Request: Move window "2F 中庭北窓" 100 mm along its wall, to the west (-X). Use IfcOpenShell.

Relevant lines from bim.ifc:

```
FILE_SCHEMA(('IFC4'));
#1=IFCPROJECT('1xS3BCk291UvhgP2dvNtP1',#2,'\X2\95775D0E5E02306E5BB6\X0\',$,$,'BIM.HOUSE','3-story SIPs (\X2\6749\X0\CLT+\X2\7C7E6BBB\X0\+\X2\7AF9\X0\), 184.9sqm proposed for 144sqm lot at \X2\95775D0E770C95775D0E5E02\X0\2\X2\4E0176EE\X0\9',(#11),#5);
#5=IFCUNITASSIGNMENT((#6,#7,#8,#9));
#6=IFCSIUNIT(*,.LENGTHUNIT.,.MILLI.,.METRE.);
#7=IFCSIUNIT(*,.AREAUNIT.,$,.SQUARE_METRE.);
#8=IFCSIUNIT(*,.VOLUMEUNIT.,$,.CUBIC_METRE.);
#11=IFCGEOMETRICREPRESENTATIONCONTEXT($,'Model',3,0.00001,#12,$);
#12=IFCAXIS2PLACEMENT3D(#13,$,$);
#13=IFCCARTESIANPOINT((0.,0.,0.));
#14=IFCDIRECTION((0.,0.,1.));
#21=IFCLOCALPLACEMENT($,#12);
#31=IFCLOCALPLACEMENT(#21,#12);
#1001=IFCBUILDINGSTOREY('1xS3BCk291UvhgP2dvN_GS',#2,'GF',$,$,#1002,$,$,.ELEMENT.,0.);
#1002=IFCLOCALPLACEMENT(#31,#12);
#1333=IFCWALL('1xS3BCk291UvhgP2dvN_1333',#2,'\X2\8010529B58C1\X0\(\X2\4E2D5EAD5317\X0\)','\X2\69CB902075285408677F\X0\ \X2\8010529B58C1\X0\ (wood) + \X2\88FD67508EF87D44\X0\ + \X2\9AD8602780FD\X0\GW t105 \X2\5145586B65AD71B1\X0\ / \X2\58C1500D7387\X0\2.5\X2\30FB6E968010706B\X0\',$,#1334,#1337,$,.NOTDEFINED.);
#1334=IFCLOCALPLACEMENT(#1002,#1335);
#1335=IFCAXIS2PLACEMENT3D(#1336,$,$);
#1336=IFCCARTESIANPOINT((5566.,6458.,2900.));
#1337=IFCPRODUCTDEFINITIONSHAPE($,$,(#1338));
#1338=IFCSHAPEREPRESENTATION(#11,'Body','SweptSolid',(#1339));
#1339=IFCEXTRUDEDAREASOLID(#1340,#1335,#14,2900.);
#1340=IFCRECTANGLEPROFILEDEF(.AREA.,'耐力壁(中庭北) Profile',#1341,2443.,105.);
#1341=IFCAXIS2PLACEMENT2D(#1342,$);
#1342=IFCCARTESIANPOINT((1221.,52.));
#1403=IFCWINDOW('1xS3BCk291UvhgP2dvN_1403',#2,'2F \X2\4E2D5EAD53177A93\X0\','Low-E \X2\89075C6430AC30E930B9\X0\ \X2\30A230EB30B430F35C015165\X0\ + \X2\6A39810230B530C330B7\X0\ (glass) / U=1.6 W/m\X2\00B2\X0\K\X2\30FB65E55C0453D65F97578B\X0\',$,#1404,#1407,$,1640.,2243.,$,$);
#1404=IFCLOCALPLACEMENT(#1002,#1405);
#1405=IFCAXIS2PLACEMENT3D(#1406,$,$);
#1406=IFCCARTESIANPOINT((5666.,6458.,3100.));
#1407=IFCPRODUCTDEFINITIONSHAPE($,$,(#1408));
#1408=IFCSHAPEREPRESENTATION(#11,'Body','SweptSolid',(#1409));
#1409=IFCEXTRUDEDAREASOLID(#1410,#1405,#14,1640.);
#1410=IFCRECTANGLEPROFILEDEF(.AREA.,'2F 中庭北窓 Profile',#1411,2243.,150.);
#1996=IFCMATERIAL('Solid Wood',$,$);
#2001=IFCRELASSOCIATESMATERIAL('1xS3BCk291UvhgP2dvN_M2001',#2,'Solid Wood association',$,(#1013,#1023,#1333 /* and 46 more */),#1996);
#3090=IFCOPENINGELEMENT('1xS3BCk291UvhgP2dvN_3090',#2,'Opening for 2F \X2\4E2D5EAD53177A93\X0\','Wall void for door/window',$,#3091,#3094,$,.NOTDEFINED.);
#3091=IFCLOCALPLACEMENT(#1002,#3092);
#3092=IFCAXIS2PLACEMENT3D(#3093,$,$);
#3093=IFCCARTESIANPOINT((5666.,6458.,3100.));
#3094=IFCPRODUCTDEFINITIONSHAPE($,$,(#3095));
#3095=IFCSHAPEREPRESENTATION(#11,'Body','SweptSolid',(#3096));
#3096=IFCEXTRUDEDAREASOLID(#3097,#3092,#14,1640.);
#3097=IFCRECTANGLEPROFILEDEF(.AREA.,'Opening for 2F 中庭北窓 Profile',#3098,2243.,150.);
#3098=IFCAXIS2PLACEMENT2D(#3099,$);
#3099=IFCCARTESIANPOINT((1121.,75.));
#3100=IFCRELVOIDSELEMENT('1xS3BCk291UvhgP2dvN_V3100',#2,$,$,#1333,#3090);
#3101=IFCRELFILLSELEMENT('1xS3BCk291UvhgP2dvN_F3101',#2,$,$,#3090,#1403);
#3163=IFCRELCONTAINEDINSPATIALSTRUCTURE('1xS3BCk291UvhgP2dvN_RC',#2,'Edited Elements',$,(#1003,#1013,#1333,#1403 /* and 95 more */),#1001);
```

```python
import ifcopenshell
import ifcopenshell.api.geometry
import ifcopenshell.util.placement
import ifcopenshell.util.unit

model = ifcopenshell.open("bim.ifc")
unit_scale = ifcopenshell.util.unit.calculate_unit_scale(model)

window = model.by_guid("1xS3BCk291UvhgP2dvN_1403")
opening = window.FillsVoids[0].RelatingOpeningElement
wall = opening.VoidsElements[0].RelatingBuildingElement

wall_matrix = ifcopenshell.util.placement.get_local_placement(wall.ObjectPlacement)
shift = wall_matrix[:3, 0] * -0.1 / unit_scale
before = ifcopenshell.util.placement.get_local_placement(window.ObjectPlacement)[:3, 3].copy()

# The window is not placed relative to its opening, so move both.
for product in (opening, window):
    matrix = ifcopenshell.util.placement.get_local_placement(product.ObjectPlacement)
    matrix[:3, 3] += shift
    ifcopenshell.api.geometry.edit_object_placement(model, product=product, matrix=matrix, is_si=False)

after = ifcopenshell.util.placement.get_local_placement(window.ObjectPlacement)[:3, 3]
print("window moved by", (after - before).round(3) + 0.0)

model.write("bim_rev.ifc")
```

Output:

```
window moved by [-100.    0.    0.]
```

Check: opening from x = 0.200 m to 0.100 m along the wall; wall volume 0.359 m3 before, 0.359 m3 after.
